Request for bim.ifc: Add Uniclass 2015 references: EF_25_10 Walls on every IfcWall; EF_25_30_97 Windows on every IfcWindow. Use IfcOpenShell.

First a look at what the model holds.

```python
import ifcopenshell

model = ifcopenshell.open("bim.ifc")
print(model.schema)
print("classifications:", [c.Name for c in model.by_type("IfcClassification")])
for ifc_class in ("IfcDoor", "IfcRoof", "IfcStair", "IfcWall", "IfcWindow"):
    print(ifc_class, len(model.by_type(ifc_class)))
```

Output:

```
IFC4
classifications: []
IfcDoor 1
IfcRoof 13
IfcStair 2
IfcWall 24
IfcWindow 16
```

```python
import ifcopenshell
import ifcopenshell.api.classification

model = ifcopenshell.open("bim.ifc")

system = ifcopenshell.api.classification.add_classification(model, classification="Uniclass 2015")

codes = {
    "IfcWall": ("EF_25_10", "Walls"),
    "IfcWindow": ("EF_25_30_97", "Windows"),
}
for ifc_class, (code, name) in codes.items():
    products = model.by_type(ifc_class)
    ifcopenshell.api.classification.add_reference(
        model, products=products, classification=system, identification=code, name=name
    )
    print(code, len(products))

model.write("bim-out.ifc")
```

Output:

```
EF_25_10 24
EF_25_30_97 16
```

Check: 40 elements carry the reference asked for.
